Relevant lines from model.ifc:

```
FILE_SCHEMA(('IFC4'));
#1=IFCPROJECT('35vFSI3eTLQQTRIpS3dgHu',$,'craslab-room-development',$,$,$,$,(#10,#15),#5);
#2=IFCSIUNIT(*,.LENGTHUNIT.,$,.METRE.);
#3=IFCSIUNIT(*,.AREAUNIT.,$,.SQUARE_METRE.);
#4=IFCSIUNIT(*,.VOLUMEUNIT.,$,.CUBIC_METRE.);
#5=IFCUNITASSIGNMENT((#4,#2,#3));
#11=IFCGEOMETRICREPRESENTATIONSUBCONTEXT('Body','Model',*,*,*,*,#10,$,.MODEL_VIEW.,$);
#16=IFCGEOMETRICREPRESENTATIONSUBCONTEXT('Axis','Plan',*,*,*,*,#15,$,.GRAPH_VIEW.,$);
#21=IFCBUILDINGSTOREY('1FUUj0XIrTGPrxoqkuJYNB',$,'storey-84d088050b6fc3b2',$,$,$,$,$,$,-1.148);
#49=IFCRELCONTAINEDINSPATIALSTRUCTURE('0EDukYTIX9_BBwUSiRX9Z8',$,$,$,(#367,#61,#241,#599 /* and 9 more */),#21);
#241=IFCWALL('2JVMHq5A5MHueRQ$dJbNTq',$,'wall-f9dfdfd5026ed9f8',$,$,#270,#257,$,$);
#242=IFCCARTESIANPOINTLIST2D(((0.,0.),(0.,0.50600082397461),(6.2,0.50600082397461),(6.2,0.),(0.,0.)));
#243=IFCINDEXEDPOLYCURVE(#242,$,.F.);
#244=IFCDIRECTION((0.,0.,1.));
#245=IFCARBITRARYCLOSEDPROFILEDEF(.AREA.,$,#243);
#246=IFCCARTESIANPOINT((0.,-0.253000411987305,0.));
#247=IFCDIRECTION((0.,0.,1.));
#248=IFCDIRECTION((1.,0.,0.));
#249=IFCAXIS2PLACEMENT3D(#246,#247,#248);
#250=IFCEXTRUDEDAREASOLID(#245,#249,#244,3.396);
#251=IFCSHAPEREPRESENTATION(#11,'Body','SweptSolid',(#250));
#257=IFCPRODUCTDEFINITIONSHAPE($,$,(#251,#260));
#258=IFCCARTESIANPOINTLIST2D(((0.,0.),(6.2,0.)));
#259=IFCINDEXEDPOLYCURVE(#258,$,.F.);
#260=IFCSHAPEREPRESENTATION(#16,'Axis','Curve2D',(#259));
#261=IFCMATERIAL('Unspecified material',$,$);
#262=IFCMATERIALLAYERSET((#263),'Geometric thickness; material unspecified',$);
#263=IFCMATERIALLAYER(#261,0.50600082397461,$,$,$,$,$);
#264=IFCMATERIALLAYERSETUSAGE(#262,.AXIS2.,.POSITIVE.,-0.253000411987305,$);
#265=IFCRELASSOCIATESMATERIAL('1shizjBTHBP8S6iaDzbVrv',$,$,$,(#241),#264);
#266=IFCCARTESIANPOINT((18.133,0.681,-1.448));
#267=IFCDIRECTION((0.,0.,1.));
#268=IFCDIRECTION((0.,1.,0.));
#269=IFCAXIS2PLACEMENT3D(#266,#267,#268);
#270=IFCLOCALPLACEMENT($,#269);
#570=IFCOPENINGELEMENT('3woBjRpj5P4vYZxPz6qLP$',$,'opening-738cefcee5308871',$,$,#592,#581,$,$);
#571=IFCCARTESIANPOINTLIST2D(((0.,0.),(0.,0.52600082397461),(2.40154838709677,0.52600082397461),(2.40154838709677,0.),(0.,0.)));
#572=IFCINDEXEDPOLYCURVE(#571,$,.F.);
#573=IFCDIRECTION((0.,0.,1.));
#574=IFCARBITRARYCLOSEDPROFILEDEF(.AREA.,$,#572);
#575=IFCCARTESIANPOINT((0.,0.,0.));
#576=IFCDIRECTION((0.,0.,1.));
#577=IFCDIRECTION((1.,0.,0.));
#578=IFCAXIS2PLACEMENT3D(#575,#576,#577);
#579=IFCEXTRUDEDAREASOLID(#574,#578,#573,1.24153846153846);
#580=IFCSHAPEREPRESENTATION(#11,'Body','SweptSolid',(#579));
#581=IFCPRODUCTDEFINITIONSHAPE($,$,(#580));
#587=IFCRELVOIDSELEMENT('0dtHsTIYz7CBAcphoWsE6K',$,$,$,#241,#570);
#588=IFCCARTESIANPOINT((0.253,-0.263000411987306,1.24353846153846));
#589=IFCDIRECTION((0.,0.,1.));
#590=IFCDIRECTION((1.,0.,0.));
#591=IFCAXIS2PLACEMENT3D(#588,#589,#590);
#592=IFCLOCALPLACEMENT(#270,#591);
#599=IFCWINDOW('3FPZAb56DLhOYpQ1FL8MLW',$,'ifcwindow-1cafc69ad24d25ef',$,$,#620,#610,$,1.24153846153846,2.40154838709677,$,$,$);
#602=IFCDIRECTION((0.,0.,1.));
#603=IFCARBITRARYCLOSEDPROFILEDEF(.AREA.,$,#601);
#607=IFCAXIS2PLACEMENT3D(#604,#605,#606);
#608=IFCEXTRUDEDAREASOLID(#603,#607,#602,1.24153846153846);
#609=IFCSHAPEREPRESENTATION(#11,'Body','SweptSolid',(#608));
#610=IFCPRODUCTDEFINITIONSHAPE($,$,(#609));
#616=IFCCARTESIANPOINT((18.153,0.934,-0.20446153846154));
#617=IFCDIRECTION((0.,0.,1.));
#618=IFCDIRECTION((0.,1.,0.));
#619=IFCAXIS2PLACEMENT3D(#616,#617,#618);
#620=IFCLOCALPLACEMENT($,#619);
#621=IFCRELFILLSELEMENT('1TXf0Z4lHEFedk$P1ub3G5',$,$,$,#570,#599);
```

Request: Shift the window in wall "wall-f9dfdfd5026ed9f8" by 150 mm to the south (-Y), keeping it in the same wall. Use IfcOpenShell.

```python
import ifcopenshell
import ifcopenshell.api.geometry
import ifcopenshell.util.placement
import ifcopenshell.util.unit

model = ifcopenshell.open("model.ifc")
unit_scale = ifcopenshell.util.unit.calculate_unit_scale(model)

window = model.by_guid("3FPZAb56DLhOYpQ1FL8MLW")
opening = window.FillsVoids[0].RelatingOpeningElement
wall = opening.VoidsElements[0].RelatingBuildingElement

wall_matrix = ifcopenshell.util.placement.get_local_placement(wall.ObjectPlacement)
shift = wall_matrix[:3, 0] * -0.15 / unit_scale
before = ifcopenshell.util.placement.get_local_placement(window.ObjectPlacement)[:3, 3].copy()

# The window is not placed relative to its opening, so move both.
for product in (opening, window):
    matrix = ifcopenshell.util.placement.get_local_placement(product.ObjectPlacement)
    matrix[:3, 3] += shift
    ifcopenshell.api.geometry.edit_object_placement(model, product=product, matrix=matrix, is_si=False)

after = ifcopenshell.util.placement.get_local_placement(window.ObjectPlacement)[:3, 3]
print("window moved by", (after - before).round(3) + 0.0)

model.write("model-out.ifc")
```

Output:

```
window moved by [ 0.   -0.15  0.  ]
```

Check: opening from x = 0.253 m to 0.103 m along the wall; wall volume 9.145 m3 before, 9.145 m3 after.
